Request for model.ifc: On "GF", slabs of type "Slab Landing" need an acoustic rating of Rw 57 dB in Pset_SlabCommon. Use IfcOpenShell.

First a look at what the model holds.

```python
import ifcopenshell
import ifcopenshell.util.element

model = ifcopenshell.open("model.ifc")
print(model.schema)
storey = next(s for s in model.by_type("IfcBuildingStorey") if s.Name == "GF")
slabs = [e for e in ifcopenshell.util.element.get_decomposition(storey) if e.is_a("IfcSlab")]
seen = {}
for e in slabs:
    element_type = ifcopenshell.util.element.get_type(e)
    key = (element_type.Name if element_type != e and element_type else None, ifcopenshell.util.element.get_pset(e, "Pset_SlabCommon", "AcousticRating"))
    seen[key] = seen.get(key, 0) + 1
for (name, value), count in sorted(seen.items(), key=str):
    print(count, "x", name, "|", value)
```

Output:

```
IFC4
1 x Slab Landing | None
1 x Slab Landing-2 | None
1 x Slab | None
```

```python
import ifcopenshell
import ifcopenshell.api.pset
import ifcopenshell.util.element

model = ifcopenshell.open("model.ifc")

storey = next(s for s in model.by_type("IfcBuildingStorey") if s.Name == "GF")
slabs = [e for e in ifcopenshell.util.element.get_decomposition(storey) if e.is_a("IfcSlab")]

count = 0
for e in slabs:
    element_type = ifcopenshell.util.element.get_type(e)
    if element_type in (None, e) or element_type.Name != "Slab Landing":
        continue
    # add_pset returns the element's existing set when there is one.
    pset = ifcopenshell.api.pset.add_pset(model, product=e, name="Pset_SlabCommon")
    ifcopenshell.api.pset.edit_pset(model, pset=pset, properties={"AcousticRating": "Rw 57 dB"})
    count += 1

print(count, "slabs updated")

model.write("model_v2.ifc")
```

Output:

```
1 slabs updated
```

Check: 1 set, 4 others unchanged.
